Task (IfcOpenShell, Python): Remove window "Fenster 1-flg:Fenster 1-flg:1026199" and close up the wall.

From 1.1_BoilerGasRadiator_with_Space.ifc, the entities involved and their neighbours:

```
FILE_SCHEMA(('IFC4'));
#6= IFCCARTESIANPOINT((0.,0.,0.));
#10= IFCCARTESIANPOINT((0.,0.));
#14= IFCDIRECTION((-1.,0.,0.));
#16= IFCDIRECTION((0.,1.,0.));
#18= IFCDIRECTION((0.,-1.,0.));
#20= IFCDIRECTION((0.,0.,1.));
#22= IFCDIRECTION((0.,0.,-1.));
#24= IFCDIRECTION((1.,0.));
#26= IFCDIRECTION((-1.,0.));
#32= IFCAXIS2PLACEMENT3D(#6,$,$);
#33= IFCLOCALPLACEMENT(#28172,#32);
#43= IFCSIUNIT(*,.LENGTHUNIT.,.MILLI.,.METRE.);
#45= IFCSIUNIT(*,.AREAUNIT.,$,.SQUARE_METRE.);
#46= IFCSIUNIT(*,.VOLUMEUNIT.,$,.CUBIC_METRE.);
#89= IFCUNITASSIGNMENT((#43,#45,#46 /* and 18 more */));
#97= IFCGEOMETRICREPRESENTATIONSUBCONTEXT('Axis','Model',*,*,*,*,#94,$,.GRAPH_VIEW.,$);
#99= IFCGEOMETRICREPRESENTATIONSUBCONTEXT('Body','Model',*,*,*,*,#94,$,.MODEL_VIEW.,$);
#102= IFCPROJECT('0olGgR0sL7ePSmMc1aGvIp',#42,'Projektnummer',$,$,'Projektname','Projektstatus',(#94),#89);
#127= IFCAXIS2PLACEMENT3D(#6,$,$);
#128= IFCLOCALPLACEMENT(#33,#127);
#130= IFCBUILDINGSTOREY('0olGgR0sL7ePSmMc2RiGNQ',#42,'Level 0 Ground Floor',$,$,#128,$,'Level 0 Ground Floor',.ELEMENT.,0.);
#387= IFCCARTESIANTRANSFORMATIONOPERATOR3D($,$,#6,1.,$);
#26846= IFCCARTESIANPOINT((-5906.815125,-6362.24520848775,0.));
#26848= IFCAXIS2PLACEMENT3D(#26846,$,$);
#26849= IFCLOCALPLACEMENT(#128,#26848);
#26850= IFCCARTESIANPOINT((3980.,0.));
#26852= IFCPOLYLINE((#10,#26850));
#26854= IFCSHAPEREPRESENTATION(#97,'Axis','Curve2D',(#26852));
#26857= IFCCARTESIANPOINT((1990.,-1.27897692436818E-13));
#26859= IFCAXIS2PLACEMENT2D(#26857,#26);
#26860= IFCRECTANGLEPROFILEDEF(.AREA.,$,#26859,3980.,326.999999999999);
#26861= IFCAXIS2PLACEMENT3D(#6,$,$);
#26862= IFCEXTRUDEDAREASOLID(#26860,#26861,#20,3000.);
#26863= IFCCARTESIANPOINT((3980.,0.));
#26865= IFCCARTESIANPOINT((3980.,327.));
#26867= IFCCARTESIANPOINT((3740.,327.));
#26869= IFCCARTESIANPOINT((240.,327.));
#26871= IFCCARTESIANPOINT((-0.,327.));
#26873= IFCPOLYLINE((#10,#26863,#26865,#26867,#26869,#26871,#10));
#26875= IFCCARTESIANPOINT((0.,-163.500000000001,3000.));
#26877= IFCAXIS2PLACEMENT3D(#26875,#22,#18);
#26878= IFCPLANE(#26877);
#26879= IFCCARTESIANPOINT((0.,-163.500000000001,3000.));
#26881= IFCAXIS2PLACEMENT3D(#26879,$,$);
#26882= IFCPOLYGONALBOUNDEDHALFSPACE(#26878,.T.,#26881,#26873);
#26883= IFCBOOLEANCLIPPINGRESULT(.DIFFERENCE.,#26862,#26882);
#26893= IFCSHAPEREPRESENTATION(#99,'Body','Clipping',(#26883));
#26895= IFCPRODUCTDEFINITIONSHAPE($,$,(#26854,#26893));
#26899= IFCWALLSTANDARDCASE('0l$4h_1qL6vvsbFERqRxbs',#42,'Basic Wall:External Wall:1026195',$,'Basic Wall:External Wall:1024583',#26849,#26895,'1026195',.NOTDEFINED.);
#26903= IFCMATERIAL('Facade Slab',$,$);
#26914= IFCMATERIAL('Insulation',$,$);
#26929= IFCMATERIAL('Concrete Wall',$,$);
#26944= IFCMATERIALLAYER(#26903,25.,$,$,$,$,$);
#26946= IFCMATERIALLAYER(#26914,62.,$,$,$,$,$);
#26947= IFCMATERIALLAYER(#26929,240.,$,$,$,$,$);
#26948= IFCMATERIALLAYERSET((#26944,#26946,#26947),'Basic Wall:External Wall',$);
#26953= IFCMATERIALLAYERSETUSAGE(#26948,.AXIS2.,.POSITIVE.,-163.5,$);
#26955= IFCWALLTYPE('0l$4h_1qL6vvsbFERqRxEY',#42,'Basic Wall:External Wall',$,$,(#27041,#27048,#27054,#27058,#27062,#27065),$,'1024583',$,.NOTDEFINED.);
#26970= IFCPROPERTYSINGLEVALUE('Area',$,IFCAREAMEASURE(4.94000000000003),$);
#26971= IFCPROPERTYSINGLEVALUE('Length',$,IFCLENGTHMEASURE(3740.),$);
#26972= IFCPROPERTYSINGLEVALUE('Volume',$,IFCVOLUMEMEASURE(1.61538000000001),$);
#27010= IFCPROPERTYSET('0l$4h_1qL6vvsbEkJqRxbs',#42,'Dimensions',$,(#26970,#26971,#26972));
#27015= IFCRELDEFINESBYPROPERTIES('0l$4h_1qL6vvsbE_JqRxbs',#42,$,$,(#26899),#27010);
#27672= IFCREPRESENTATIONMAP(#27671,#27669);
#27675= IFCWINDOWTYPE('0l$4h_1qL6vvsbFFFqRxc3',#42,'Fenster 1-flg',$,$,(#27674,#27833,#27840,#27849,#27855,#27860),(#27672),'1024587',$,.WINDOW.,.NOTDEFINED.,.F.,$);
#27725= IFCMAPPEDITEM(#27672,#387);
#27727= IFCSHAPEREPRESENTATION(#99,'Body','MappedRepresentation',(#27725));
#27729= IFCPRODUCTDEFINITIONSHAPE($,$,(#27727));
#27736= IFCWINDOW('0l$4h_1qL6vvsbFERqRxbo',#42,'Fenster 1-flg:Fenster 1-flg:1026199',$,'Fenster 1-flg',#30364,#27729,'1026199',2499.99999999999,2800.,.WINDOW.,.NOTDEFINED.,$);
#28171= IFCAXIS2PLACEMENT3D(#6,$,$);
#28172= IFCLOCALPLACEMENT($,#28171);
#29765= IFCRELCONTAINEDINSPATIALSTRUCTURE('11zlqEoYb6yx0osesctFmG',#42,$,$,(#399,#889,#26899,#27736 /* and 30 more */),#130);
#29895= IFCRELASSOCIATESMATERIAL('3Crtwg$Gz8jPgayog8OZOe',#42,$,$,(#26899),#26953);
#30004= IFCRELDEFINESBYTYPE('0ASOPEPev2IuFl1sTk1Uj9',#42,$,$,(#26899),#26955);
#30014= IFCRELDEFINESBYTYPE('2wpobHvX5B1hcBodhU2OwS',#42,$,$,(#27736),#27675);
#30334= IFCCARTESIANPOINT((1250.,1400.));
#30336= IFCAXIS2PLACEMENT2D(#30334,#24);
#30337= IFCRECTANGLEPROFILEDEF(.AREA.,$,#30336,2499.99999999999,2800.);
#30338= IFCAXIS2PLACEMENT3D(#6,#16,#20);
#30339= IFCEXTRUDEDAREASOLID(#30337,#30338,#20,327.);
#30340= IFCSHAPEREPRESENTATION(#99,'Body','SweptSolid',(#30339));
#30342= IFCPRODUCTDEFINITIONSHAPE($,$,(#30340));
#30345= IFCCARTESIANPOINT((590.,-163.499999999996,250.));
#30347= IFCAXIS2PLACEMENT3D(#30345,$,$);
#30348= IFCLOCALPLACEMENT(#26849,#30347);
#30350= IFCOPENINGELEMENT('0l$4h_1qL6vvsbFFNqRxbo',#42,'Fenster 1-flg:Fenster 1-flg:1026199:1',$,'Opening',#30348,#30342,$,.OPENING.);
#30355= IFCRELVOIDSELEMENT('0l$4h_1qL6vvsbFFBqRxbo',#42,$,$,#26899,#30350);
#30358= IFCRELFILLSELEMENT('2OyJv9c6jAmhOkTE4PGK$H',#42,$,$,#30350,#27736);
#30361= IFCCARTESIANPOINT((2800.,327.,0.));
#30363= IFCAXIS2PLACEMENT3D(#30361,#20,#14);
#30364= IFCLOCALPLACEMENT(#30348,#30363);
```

```python
import ifcopenshell
import ifcopenshell.api.feature
import ifcopenshell.api.pset
import ifcopenshell.api.root
import ifcopenshell.geom
import ifcopenshell.util.element
import ifcopenshell.util.shape
import ifcopenshell.util.unit

model = ifcopenshell.open("1.1_BoilerGasRadiator_with_Space.ifc")
area_scale = ifcopenshell.util.unit.calculate_unit_scale(model, "AREAUNIT")
volume_scale = ifcopenshell.util.unit.calculate_unit_scale(model, "VOLUMEUNIT")
settings = ifcopenshell.geom.settings()


def volume(element):
    """Net volume in cubic metres, openings subtracted."""
    shape = ifcopenshell.geom.create_shape(settings, element)
    return ifcopenshell.util.shape.get_volume(shape.geometry)


window = model.by_guid("0l$4h_1qL6vvsbFERqRxbo")
opening = window.FillsVoids[0].RelatingOpeningElement
wall = opening.VoidsElements[0].RelatingBuildingElement
before = volume(wall)

ifcopenshell.api.root.remove_product(model, product=window)
ifcopenshell.api.feature.remove_feature(model, feature=opening)

after = volume(wall)
thickness = 0.327  # wall thickness in metres

# Update the wall's stored quantities.
pset = model.by_id(ifcopenshell.util.element.get_pset(wall, "Dimensions", should_inherit=False)["id"])
ifcopenshell.api.pset.edit_pset(model, pset=pset, properties={
    "Area": model.create_entity("IfcAreaMeasure", after / thickness / area_scale),
    "Volume": model.create_entity("IfcVolumeMeasure", after / volume_scale),
})

print(f"wall volume {before:.3f} -> {after:.3f} m3")

model.write("1.1_BoilerGasRadiator_with_Space-out.ifc")
```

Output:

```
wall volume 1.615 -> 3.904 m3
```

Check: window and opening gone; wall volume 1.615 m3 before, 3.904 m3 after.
